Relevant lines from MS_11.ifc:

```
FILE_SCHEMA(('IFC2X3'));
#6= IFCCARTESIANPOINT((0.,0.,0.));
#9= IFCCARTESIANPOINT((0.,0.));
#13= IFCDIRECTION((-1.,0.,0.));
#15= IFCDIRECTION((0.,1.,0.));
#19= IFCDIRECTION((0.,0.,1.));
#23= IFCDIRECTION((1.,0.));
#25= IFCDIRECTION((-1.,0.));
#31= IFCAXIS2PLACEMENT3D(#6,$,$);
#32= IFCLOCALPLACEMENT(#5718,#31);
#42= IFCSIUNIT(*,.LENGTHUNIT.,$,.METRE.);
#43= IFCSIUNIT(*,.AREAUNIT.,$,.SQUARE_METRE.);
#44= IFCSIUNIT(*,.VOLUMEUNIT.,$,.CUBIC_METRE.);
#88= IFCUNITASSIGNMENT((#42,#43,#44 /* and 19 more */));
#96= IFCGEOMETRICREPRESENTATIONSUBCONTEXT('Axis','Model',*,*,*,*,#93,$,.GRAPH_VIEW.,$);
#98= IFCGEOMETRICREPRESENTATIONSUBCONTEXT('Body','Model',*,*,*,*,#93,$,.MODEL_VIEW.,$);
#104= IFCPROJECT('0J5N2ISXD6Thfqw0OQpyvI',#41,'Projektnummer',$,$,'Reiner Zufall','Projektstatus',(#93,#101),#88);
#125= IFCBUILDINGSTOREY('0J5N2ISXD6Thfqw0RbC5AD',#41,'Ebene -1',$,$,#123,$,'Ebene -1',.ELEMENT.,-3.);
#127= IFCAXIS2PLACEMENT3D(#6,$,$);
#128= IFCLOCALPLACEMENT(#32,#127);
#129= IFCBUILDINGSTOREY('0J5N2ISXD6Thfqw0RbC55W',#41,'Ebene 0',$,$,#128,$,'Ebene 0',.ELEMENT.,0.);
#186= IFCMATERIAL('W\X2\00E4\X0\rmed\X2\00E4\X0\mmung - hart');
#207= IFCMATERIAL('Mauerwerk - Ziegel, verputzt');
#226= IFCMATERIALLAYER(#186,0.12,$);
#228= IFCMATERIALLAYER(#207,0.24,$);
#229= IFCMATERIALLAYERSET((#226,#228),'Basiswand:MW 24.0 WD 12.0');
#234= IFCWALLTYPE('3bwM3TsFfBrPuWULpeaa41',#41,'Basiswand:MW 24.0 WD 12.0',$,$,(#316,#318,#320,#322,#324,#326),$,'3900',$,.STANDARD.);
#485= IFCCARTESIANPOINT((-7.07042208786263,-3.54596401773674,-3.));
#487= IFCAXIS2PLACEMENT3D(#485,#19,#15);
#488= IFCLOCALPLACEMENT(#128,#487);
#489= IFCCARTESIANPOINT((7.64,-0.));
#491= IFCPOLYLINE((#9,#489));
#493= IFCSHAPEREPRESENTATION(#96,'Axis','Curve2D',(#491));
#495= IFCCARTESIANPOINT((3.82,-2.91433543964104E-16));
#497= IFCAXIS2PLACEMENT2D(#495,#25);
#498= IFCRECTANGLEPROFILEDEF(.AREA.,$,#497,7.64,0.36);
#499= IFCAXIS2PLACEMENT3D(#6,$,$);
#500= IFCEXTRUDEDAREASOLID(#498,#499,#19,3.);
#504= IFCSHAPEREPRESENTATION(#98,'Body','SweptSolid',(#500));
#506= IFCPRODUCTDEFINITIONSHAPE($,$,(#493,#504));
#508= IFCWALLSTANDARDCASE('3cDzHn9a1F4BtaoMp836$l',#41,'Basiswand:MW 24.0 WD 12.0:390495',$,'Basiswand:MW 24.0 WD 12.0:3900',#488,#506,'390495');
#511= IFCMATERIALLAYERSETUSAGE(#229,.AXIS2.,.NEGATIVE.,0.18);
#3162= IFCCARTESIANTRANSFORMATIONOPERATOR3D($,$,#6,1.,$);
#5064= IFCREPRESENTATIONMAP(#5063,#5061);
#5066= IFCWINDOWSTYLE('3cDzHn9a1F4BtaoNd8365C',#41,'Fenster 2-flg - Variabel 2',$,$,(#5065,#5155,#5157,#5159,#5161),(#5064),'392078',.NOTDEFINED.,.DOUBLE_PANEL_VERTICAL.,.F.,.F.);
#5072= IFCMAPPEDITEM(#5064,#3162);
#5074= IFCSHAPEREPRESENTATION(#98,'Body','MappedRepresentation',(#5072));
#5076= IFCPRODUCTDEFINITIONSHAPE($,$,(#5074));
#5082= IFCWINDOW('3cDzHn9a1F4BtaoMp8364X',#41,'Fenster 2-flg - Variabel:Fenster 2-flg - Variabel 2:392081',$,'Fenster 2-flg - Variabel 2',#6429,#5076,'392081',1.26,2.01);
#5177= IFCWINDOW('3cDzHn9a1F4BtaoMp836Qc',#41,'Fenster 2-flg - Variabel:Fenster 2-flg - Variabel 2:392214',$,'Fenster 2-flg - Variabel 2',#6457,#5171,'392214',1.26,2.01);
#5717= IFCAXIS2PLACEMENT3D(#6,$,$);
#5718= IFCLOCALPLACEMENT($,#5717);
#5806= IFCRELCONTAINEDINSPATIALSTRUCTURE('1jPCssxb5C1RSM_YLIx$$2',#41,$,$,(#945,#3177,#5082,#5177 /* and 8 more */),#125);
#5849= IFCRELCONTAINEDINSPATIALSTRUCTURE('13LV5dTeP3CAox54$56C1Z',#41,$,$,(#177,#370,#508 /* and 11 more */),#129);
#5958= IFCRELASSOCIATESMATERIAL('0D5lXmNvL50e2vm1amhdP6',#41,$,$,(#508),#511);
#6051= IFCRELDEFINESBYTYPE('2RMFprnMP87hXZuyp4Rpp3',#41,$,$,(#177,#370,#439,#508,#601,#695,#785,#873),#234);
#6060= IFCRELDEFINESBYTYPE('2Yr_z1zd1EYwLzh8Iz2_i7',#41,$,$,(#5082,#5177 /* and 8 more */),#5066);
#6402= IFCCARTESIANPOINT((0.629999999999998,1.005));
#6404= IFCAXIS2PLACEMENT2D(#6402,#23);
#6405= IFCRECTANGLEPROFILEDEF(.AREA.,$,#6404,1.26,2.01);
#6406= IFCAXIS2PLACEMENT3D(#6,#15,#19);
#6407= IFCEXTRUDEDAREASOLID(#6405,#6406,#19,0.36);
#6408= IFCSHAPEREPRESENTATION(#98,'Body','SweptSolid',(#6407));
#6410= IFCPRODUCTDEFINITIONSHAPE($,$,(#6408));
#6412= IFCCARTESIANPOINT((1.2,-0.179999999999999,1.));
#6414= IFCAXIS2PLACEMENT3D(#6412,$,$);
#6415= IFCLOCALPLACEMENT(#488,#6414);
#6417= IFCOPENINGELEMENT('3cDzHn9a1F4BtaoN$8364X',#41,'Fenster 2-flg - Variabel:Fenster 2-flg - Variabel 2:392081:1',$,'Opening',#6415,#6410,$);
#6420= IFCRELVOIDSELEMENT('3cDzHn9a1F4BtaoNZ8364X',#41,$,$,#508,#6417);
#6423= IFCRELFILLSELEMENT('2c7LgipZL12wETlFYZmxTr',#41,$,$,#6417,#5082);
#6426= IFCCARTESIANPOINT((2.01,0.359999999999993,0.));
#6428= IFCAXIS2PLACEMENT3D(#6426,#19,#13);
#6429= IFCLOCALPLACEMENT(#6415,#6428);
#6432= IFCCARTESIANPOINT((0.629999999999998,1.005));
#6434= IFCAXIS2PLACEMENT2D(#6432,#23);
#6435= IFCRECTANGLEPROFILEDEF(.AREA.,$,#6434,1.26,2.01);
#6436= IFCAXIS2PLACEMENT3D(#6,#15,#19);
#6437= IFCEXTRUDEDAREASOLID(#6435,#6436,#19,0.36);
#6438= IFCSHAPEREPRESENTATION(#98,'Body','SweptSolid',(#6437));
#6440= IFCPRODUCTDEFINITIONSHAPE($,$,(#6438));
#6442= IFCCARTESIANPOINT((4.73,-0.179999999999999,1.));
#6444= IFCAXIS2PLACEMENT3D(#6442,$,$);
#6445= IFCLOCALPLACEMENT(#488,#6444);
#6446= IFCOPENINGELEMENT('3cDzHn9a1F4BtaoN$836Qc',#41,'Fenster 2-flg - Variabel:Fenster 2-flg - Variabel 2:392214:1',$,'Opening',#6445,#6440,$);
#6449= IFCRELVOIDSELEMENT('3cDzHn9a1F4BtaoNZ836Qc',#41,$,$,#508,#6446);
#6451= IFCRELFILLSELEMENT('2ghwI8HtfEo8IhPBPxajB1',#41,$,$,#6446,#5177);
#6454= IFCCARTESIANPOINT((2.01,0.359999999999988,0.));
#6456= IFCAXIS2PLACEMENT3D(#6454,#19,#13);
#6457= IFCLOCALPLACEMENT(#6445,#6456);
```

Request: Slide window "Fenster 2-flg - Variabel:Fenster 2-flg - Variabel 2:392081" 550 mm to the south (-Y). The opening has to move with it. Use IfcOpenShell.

```python
import ifcopenshell
import ifcopenshell.api.geometry
import ifcopenshell.util.placement
import ifcopenshell.util.unit

model = ifcopenshell.open("MS_11.ifc")
unit_scale = ifcopenshell.util.unit.calculate_unit_scale(model)

window = model.by_guid("3cDzHn9a1F4BtaoMp8364X")
opening = window.FillsVoids[0].RelatingOpeningElement
wall = opening.VoidsElements[0].RelatingBuildingElement

wall_matrix = ifcopenshell.util.placement.get_local_placement(wall.ObjectPlacement)
shift = wall_matrix[:3, 0] * -0.55 / unit_scale
before = ifcopenshell.util.placement.get_local_placement(window.ObjectPlacement)[:3, 3].copy()

# The window is placed relative to its opening, so it follows when the opening moves.
matrix = ifcopenshell.util.placement.get_local_placement(opening.ObjectPlacement)
matrix[:3, 3] += shift
ifcopenshell.api.geometry.edit_object_placement(
    model, product=opening, matrix=matrix, is_si=False, should_transform_children=True
)

after = ifcopenshell.util.placement.get_local_placement(window.ObjectPlacement)[:3, 3]
print("window moved by", (after - before).round(3) + 0.0)

model.write("MS_11_updated.ifc")
```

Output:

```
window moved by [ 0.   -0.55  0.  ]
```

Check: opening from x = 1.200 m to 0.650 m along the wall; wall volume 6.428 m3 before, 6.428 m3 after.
